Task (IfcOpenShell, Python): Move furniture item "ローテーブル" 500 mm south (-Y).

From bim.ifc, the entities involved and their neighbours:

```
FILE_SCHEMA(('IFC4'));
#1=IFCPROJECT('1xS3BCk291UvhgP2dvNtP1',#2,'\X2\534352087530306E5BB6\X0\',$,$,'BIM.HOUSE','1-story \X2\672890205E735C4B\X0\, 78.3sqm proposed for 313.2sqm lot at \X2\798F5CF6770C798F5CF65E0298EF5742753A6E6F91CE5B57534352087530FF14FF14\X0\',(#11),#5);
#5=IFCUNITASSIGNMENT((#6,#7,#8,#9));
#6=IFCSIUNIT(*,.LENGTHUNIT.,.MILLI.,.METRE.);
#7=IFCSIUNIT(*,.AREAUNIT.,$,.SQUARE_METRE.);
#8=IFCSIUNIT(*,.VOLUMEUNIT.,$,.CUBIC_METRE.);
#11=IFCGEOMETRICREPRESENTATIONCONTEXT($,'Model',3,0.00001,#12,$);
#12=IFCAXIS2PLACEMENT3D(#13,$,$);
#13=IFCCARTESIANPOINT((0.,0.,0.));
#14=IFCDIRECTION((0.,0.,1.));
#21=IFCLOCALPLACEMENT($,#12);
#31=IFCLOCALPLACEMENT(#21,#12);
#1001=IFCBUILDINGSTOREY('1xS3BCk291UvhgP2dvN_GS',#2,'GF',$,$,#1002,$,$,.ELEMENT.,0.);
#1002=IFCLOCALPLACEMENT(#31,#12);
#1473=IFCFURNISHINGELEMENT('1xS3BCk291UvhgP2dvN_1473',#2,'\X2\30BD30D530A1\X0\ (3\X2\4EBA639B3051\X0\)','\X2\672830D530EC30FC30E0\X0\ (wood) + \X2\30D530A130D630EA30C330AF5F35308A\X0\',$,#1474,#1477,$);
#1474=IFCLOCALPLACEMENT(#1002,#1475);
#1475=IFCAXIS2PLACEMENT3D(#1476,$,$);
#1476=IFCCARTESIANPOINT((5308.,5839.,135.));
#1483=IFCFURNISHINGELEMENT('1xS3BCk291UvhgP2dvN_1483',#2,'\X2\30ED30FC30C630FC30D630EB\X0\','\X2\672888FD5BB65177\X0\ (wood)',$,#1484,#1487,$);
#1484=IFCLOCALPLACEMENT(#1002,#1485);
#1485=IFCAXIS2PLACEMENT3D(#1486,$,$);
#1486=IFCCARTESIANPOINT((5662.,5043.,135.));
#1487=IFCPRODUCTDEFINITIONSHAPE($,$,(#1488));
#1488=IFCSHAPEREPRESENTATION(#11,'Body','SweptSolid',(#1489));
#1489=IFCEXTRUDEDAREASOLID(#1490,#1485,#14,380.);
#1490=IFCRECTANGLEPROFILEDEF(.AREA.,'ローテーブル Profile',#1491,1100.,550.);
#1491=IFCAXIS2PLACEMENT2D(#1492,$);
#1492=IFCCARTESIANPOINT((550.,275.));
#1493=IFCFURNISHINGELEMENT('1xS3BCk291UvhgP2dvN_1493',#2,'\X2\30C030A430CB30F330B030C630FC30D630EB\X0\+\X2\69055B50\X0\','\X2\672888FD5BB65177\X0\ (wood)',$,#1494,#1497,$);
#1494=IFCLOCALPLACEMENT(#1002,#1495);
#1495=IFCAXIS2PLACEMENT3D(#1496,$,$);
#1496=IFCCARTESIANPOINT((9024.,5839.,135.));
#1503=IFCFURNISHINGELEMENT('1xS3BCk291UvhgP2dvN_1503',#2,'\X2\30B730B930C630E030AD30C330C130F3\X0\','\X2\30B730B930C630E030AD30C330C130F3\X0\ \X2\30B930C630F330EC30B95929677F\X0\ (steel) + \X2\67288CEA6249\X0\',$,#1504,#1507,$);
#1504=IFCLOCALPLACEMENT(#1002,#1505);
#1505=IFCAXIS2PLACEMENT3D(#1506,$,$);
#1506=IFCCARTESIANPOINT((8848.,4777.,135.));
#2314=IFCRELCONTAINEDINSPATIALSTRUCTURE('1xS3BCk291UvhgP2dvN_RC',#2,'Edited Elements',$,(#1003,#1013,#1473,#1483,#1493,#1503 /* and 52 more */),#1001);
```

```python
import ifcopenshell
import ifcopenshell.api.geometry
import ifcopenshell.util.placement
import ifcopenshell.util.unit

model = ifcopenshell.open("bim.ifc")
unit_scale = ifcopenshell.util.unit.calculate_unit_scale(model)

item = model.by_id(1483)
matrix = ifcopenshell.util.placement.get_local_placement(item.ObjectPlacement)
matrix[1, 3] -= 0.5 / unit_scale
ifcopenshell.api.geometry.edit_object_placement(model, product=item, matrix=matrix, is_si=False)

print(ifcopenshell.util.placement.get_local_placement(item.ObjectPlacement).round(3) + 0.0)

model.write("bim_updated.ifc")
```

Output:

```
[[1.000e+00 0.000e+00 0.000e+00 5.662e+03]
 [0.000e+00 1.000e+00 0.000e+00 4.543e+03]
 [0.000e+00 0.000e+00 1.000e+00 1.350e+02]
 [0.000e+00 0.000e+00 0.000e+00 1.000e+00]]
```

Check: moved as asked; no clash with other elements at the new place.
